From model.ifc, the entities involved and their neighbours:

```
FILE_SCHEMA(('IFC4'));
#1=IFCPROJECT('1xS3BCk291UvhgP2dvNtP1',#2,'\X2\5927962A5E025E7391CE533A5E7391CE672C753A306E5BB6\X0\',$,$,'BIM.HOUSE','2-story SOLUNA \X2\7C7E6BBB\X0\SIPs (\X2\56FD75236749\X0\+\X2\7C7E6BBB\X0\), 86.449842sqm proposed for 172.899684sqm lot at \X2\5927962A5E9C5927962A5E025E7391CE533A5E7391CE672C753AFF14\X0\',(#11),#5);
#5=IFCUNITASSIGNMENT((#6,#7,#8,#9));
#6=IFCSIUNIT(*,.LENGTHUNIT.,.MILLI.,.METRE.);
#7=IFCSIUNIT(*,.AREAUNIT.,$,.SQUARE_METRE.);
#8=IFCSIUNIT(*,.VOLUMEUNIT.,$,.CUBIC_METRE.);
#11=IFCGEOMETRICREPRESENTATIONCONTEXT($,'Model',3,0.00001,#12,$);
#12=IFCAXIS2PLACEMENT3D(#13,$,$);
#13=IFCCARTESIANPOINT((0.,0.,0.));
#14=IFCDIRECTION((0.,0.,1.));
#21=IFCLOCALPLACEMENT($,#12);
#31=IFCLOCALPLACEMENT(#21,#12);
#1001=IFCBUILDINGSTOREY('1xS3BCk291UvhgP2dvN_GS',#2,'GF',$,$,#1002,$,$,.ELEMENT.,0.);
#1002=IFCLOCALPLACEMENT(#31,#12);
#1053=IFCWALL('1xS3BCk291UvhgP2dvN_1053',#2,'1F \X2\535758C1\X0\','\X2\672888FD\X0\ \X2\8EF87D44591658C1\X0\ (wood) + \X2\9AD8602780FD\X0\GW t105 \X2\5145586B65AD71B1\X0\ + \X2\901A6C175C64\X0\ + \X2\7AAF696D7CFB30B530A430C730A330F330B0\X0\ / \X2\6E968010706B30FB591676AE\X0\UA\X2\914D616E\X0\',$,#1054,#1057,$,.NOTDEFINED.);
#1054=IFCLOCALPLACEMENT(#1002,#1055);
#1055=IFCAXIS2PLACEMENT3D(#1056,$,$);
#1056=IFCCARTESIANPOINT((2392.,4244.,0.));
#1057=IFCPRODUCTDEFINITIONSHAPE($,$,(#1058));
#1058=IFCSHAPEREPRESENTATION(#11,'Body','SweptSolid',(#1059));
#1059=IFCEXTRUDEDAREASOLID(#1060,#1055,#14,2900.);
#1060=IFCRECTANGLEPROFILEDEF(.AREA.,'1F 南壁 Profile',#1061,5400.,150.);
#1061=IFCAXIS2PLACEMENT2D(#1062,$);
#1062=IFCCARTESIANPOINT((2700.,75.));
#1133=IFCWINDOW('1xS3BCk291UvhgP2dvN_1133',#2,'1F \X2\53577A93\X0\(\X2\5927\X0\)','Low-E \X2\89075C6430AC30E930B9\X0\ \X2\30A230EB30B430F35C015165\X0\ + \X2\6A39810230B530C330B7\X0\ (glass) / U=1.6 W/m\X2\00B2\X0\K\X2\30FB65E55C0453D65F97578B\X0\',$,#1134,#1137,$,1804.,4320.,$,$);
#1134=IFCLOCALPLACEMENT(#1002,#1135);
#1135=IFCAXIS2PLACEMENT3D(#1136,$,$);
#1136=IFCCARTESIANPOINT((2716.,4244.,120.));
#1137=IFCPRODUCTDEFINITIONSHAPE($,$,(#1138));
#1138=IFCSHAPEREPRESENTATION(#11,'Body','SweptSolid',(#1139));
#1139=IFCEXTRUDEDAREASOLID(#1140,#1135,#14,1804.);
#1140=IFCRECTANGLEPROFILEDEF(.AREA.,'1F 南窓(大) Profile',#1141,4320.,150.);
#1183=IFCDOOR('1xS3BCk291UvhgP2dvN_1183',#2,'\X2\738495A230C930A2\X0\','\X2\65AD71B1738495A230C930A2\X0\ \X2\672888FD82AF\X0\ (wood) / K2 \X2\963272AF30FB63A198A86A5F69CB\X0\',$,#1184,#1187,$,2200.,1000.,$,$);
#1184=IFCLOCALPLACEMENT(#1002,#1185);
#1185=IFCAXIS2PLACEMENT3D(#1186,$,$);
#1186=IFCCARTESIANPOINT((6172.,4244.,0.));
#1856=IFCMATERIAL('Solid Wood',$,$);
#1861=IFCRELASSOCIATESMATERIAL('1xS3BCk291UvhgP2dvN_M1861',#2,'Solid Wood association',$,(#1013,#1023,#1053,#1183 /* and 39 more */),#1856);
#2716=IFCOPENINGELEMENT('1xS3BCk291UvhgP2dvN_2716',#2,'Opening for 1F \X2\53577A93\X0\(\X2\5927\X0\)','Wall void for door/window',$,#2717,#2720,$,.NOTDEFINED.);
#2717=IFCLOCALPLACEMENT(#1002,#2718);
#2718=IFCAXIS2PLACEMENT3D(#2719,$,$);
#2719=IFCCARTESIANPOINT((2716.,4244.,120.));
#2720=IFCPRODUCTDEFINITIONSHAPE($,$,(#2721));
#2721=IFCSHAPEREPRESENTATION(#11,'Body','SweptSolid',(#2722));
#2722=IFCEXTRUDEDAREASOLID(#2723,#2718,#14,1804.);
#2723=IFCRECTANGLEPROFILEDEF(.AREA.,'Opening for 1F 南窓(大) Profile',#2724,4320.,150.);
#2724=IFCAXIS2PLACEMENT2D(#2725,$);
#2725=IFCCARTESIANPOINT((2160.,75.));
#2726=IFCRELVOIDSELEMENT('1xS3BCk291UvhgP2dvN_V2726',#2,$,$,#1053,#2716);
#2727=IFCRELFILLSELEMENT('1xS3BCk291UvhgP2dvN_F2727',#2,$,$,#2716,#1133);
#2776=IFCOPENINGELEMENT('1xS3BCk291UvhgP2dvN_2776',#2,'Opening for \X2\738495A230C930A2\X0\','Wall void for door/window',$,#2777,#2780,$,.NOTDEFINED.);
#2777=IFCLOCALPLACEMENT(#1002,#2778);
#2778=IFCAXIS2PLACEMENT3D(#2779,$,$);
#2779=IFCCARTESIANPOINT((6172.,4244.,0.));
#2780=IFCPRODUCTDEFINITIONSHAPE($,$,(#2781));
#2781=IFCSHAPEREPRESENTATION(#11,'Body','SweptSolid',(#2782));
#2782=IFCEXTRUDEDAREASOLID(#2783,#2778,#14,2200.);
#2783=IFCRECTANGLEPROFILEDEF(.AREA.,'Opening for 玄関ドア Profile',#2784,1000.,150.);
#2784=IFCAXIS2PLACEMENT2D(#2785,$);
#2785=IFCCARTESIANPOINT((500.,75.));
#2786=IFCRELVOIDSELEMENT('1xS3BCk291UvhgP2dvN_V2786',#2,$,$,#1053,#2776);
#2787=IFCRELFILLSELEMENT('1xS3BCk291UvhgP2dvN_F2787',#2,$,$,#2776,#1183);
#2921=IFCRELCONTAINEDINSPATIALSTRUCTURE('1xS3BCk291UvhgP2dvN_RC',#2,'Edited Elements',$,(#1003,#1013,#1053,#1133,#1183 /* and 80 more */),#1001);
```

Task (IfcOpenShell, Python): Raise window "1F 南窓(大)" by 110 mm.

```python
import numpy as np
import ifcopenshell
import ifcopenshell.api.geometry
import ifcopenshell.util.placement
import ifcopenshell.util.unit

model = ifcopenshell.open("model.ifc")
unit_scale = ifcopenshell.util.unit.calculate_unit_scale(model)

window = model.by_id(1133)
opening = window.FillsVoids[0].RelatingOpeningElement
dz = 110.0

shift = np.array([0.0, 0.0, dz])
# The window is not placed relative to its opening, so move both.
for product in (opening, window):
    matrix = ifcopenshell.util.placement.get_local_placement(product.ObjectPlacement)
    matrix[:3, 3] += shift
    ifcopenshell.api.geometry.edit_object_placement(model, product=product, matrix=matrix, is_si=False)

print(f"moved by {dz * unit_scale:+.3f} m")

model.write("model_v2.ifc")
```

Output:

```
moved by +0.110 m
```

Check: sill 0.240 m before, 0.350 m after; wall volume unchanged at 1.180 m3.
